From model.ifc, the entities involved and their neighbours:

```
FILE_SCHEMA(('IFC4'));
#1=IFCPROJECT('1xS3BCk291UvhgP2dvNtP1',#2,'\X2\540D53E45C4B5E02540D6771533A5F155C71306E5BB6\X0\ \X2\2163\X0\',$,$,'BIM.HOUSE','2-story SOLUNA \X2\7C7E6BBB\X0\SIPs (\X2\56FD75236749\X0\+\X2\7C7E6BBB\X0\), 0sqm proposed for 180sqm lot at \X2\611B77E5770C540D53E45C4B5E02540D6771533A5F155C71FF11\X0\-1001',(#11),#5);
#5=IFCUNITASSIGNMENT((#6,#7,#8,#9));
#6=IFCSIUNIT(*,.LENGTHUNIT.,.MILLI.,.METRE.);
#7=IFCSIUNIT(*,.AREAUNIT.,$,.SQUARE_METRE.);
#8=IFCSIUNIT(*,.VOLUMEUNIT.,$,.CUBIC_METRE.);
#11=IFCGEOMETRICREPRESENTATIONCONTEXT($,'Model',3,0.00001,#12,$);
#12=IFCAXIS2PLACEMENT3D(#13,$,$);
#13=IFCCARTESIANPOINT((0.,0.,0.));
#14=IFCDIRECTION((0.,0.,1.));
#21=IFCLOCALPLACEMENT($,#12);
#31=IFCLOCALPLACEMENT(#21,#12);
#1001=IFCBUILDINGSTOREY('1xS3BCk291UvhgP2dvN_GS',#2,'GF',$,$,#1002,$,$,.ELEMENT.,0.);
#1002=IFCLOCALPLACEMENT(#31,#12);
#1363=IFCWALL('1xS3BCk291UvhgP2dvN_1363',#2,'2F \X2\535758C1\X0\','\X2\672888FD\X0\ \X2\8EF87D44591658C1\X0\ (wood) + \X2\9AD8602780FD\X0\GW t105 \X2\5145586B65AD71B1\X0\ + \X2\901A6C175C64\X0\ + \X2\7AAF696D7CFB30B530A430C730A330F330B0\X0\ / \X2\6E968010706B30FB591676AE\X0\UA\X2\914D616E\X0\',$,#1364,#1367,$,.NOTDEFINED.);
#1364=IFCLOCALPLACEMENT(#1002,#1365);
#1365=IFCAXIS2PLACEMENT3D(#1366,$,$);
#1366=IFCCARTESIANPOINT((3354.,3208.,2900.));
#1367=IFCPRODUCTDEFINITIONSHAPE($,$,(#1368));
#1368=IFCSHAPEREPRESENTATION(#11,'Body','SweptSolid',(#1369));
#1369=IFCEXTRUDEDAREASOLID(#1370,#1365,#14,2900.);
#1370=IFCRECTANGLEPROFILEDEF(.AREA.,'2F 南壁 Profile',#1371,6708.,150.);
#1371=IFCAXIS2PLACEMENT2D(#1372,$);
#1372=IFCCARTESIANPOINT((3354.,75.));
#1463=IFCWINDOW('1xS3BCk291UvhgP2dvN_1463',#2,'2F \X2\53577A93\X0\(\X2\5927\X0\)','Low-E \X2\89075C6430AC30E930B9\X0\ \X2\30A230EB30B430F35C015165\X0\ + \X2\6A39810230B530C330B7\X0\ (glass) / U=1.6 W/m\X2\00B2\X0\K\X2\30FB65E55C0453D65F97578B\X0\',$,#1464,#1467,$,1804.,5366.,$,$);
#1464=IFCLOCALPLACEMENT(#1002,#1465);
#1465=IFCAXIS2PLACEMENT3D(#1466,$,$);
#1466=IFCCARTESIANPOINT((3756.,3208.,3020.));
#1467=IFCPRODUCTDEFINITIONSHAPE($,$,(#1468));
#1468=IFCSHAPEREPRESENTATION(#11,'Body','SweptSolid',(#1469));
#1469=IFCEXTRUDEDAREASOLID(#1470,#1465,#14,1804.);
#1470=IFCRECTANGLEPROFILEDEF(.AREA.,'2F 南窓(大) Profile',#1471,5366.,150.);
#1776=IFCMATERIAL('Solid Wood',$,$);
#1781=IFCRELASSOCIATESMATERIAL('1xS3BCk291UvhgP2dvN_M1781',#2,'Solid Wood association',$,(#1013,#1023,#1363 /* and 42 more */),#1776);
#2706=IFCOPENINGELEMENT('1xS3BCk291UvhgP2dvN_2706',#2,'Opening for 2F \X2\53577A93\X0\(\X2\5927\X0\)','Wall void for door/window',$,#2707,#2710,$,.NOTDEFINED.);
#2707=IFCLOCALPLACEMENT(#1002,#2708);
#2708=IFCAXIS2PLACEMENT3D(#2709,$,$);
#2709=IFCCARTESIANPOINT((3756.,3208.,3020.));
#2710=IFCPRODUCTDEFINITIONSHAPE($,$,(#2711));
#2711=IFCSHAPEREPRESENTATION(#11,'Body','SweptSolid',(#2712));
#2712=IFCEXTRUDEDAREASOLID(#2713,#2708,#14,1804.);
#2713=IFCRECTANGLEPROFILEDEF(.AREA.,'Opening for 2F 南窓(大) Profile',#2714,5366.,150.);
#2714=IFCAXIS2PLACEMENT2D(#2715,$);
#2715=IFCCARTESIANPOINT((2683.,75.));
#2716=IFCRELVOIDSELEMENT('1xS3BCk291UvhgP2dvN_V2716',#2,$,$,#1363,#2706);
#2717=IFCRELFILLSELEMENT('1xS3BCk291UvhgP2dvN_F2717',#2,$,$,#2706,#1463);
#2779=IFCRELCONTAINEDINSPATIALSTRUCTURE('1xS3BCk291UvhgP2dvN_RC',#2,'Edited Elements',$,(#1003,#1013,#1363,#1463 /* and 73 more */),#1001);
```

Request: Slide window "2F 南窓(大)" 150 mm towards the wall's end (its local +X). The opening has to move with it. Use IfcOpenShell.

```python
import ifcopenshell
import ifcopenshell.api.geometry
import ifcopenshell.util.placement
import ifcopenshell.util.unit

model = ifcopenshell.open("model.ifc")
unit_scale = ifcopenshell.util.unit.calculate_unit_scale(model)

window = model.by_guid("1xS3BCk291UvhgP2dvN_1463")
opening = window.FillsVoids[0].RelatingOpeningElement
wall = opening.VoidsElements[0].RelatingBuildingElement

wall_matrix = ifcopenshell.util.placement.get_local_placement(wall.ObjectPlacement)
shift = wall_matrix[:3, 0] * 0.15 / unit_scale
before = ifcopenshell.util.placement.get_local_placement(window.ObjectPlacement)[:3, 3].copy()

# The window is not placed relative to its opening, so move both.
for product in (opening, window):
    matrix = ifcopenshell.util.placement.get_local_placement(product.ObjectPlacement)
    matrix[:3, 3] += shift
    ifcopenshell.api.geometry.edit_object_placement(model, product=product, matrix=matrix, is_si=False)

after = ifcopenshell.util.placement.get_local_placement(window.ObjectPlacement)[:3, 3]
print("window moved by", (after - before).round(3) + 0.0)

model.write("model-out.ifc")
```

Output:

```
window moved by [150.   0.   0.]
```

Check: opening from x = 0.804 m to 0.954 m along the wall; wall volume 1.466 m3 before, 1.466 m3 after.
